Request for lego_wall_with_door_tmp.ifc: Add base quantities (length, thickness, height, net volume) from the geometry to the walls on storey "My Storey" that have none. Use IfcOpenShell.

First a look at what the model holds.

```python
import ifcopenshell
import ifcopenshell.util.element
import ifcopenshell.util.unit

model = ifcopenshell.open("lego_wall_with_door_tmp.ifc")
print(model.schema)
for unit_type in ("LENGTHUNIT", "AREAUNIT", "VOLUMEUNIT"):
    print(unit_type, ifcopenshell.util.unit.calculate_unit_scale(model, unit_type))
storey = next(s for s in model.by_type("IfcBuildingStorey") if s.Name == "My Storey")
walls = [e for e in ifcopenshell.util.element.get_decomposition(storey) if e.is_a("IfcWall")]
for e in sorted(walls, key=lambda e: e.id()):
    print(e.id(), e.is_a(), e.Name, list(ifcopenshell.util.element.get_psets(e, qtos_only=True)), sep=" | ")
```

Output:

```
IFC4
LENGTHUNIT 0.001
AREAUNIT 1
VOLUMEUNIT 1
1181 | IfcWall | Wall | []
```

```python
import ifcopenshell
import ifcopenshell.api.pset
import ifcopenshell.geom
import ifcopenshell.util.element
import ifcopenshell.util.shape
import ifcopenshell.util.unit

model = ifcopenshell.open("lego_wall_with_door_tmp.ifc")
unit_scale = ifcopenshell.util.unit.calculate_unit_scale(model)
volume_scale = ifcopenshell.util.unit.calculate_unit_scale(model, "VOLUMEUNIT")
settings = ifcopenshell.geom.settings()

storey = next(s for s in model.by_type("IfcBuildingStorey") if s.Name == "My Storey")
walls = [e for e in ifcopenshell.util.element.get_decomposition(storey) if e.is_a("IfcWall")]

for e in sorted(walls, key=lambda e: e.id()):
    if ifcopenshell.util.element.get_psets(e, qtos_only=True, should_inherit=False):
        continue
    # Geometry comes back in metres, in the element's own axes.
    shape = ifcopenshell.geom.create_shape(settings, e)
    values = {
        "Length": ifcopenshell.util.shape.get_x(shape.geometry) / unit_scale,
        "Width": ifcopenshell.util.shape.get_y(shape.geometry) / unit_scale,
        "Height": ifcopenshell.util.shape.get_z(shape.geometry) / unit_scale,
        "NetVolume": ifcopenshell.util.shape.get_volume(shape.geometry) / volume_scale,
    }
    qto = ifcopenshell.api.pset.add_qto(model, product=e, name="Qto_WallBaseQuantities")
    ifcopenshell.api.pset.edit_qto(model, qto=qto, properties=values)
    print(e.id(), {k: round(v, 3) for k, v in values.items()})

model.write("lego_wall_with_door_tmp_v2.ifc")
```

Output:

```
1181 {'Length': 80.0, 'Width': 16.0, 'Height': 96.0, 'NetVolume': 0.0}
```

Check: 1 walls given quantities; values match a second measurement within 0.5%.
